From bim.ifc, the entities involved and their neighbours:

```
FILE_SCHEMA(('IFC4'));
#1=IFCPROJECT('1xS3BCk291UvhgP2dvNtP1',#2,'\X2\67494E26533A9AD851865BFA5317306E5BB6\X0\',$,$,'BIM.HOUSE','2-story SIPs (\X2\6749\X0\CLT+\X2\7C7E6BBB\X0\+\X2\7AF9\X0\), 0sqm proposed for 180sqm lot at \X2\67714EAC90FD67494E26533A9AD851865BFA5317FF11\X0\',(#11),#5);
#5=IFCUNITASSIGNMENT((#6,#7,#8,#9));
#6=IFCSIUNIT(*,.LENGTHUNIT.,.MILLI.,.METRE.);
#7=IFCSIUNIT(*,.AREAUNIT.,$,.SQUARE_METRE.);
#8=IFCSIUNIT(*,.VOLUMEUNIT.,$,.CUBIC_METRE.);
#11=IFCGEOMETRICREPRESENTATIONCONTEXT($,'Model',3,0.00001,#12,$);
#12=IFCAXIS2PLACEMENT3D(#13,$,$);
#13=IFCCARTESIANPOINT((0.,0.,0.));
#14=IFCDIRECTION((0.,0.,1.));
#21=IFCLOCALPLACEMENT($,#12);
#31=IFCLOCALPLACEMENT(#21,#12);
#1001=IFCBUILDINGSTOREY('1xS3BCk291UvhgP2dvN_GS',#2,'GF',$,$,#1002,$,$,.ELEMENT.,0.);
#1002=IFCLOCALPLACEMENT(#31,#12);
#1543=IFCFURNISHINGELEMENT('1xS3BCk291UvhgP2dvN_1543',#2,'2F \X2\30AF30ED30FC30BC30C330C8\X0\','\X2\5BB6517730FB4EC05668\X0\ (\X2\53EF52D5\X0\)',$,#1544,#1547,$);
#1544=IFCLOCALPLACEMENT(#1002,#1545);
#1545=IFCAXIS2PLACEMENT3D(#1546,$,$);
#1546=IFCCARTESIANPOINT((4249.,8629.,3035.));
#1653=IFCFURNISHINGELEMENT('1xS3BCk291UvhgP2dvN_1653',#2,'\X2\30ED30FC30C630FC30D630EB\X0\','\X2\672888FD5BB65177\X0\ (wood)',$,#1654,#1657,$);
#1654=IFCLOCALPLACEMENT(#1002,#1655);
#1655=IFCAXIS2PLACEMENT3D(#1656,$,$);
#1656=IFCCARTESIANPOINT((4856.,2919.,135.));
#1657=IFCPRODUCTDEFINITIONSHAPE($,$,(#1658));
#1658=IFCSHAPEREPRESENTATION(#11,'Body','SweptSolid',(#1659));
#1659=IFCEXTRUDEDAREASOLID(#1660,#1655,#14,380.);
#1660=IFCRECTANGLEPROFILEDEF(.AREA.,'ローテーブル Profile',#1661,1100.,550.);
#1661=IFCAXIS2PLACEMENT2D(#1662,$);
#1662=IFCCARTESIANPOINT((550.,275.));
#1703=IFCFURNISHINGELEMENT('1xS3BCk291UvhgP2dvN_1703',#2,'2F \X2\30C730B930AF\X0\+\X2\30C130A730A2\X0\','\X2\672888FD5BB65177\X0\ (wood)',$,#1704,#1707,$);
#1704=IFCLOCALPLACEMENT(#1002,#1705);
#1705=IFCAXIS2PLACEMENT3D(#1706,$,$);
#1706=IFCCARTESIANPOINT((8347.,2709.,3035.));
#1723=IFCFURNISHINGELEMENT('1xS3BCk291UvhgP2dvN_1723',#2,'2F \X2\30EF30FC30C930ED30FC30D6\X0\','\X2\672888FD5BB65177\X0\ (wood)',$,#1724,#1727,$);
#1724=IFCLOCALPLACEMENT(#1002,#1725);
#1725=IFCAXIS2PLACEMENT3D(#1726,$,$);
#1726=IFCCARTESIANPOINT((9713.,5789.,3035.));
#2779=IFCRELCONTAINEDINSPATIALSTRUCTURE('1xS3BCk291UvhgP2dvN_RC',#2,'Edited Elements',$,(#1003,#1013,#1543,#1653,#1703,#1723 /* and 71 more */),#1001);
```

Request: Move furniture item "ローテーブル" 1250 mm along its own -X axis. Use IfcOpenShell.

```python
import ifcopenshell
import ifcopenshell.api.geometry
import ifcopenshell.util.placement

model = ifcopenshell.open("bim.ifc")

item = model.by_id(1653)
matrix = ifcopenshell.util.placement.get_local_placement(item.ObjectPlacement)
matrix[:3, 3] -= matrix[:3, 0] * 1250.0
ifcopenshell.api.geometry.edit_object_placement(model, product=item, matrix=matrix, is_si=False)

print(ifcopenshell.util.placement.get_local_placement(item.ObjectPlacement).round(3) + 0.0)

model.write("bim_rev.ifc")
```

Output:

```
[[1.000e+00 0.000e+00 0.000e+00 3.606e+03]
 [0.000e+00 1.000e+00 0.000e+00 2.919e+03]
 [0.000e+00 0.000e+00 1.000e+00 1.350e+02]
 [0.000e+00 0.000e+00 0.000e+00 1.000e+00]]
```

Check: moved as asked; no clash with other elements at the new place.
